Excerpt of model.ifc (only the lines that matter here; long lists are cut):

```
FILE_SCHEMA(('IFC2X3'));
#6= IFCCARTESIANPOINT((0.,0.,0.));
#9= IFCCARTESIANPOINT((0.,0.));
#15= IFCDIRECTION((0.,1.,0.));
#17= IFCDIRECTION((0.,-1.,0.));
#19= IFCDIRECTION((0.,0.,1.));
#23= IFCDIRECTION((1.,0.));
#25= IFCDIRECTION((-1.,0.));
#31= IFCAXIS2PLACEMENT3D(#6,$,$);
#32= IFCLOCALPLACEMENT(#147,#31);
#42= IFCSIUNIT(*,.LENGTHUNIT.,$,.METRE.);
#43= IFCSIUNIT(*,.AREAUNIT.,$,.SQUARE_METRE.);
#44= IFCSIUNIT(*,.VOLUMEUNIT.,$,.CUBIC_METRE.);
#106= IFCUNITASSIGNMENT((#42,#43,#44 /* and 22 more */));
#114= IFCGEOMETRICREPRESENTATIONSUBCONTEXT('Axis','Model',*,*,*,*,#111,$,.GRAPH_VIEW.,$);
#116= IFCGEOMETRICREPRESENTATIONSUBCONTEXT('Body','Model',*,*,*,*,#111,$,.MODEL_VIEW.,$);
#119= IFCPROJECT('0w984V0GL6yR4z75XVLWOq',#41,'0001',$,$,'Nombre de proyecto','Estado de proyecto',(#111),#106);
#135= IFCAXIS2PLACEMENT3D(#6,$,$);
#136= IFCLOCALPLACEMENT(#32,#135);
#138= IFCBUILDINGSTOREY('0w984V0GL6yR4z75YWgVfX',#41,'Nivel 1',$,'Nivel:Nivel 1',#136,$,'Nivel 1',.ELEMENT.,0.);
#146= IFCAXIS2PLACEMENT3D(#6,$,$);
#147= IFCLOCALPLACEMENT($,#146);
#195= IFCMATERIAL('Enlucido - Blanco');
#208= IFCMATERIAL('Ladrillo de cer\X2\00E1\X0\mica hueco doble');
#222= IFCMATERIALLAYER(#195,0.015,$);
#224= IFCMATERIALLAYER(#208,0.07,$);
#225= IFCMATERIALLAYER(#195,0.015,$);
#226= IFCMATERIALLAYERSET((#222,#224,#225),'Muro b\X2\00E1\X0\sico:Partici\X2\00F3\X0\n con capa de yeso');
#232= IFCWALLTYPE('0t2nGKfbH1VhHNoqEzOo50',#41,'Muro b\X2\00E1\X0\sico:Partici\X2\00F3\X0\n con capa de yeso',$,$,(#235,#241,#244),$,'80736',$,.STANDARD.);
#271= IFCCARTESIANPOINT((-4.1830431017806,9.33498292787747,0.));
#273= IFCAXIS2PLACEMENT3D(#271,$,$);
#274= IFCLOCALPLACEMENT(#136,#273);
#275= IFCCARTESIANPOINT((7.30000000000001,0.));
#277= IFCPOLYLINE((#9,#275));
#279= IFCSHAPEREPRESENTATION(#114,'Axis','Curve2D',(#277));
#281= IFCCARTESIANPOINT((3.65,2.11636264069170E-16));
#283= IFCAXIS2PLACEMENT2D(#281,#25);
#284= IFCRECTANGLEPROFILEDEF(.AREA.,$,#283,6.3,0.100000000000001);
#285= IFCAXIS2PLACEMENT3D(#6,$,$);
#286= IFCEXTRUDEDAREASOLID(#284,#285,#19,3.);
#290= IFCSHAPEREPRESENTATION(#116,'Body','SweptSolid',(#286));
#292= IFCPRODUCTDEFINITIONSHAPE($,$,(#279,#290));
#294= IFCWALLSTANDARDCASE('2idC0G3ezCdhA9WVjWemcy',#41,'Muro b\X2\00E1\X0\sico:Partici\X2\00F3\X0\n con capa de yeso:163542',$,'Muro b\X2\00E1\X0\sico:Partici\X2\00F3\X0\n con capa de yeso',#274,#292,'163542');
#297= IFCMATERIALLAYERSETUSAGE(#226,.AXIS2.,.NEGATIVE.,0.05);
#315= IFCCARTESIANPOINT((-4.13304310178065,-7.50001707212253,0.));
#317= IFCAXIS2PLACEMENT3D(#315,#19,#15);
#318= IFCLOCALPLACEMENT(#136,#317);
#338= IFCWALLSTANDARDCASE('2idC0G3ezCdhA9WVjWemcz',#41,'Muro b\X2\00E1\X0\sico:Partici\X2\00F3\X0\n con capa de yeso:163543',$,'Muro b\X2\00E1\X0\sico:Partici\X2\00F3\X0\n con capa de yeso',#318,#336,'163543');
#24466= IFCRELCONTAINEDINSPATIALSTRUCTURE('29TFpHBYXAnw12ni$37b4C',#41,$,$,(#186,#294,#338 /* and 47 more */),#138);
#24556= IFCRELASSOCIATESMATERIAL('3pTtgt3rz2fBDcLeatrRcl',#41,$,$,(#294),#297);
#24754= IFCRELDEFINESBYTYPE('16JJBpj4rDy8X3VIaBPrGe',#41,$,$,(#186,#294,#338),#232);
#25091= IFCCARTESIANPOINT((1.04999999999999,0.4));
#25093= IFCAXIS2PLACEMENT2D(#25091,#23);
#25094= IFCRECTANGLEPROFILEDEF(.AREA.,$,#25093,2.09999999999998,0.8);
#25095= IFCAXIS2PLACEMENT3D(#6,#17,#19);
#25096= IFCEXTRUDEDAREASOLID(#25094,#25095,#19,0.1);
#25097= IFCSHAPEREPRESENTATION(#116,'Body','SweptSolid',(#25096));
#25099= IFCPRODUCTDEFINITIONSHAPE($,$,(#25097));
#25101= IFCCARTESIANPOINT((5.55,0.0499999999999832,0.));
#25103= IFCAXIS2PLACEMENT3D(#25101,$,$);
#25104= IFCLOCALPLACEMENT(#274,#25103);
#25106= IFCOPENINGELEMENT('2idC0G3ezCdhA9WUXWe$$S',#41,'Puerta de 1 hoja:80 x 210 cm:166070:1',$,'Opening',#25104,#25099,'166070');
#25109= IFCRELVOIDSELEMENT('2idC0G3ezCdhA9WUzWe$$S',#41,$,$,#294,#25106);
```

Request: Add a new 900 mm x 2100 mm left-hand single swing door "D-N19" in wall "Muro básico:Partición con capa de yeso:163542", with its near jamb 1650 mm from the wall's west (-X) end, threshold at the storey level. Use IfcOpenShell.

```python
import numpy as np
import ifcopenshell
import ifcopenshell.api.feature
import ifcopenshell.api.geometry
import ifcopenshell.api.root
import ifcopenshell.api.spatial
import ifcopenshell.api.type
import ifcopenshell.geom
import ifcopenshell.util.element
import ifcopenshell.util.placement
import ifcopenshell.util.representation
import ifcopenshell.util.shape
import ifcopenshell.util.unit

model = ifcopenshell.open("model.ifc")
unit_scale = ifcopenshell.util.unit.calculate_unit_scale(model)
settings = ifcopenshell.geom.settings()


def volume(element):
    """Net volume in cubic metres, openings subtracted."""
    shape = ifcopenshell.geom.create_shape(settings, element)
    return ifcopenshell.util.shape.get_volume(shape.geometry)


wall = model.by_guid("2idC0G3ezCdhA9WVjWemcy")
storey = ifcopenshell.util.element.get_container(wall, ifc_class="IfcBuildingStorey")
context = ifcopenshell.util.representation.get_context(model, "Model", "Body", "MODEL_VIEW")
before = volume(wall)

width, height, from_end, sill = 0.9, 2.1, 1.65, 0.0  # metres

# The wall runs along its own X axis, and the end named is its -X end.
wall_shape = ifcopenshell.geom.create_shape(settings, wall)
x, y, z = ifcopenshell.util.shape.get_vertices(wall_shape.geometry).T
start = x.min() + from_end
face, thickness = float(y.min()), float(y.max() - y.min())
wall_matrix = ifcopenshell.util.placement.get_local_placement(wall.ObjectPlacement)
level = ifcopenshell.util.placement.get_local_placement(storey.ObjectPlacement)[2, 3]


def in_wall(x, y):
    """Placement at x, y metres in the wall's axes, at sill height."""
    matrix = wall_matrix.copy()
    matrix[:, 3] = wall_matrix @ np.array([x / unit_scale, y / unit_scale, 0.0, 1.0])
    matrix[2, 3] = level + sill / unit_scale
    return matrix


# Opening: a box that overshoots both wall faces by 50 mm.
opening = ifcopenshell.api.root.create_entity(model, ifc_class="IfcOpeningElement")
box = ifcopenshell.api.geometry.add_wall_representation(
    model, context=context, length=width, height=height, thickness=thickness + 0.1
)
ifcopenshell.api.geometry.assign_representation(model, product=opening, representation=box)
ifcopenshell.api.geometry.edit_object_placement(model, product=opening, matrix=in_wall(start, face - 0.05), is_si=False)
ifcopenshell.api.feature.add_feature(model, feature=opening, element=wall)

door = ifcopenshell.api.root.create_entity(model, ifc_class="IfcDoor", name="D-N19")
door.OverallWidth, door.OverallHeight = width / unit_scale, height / unit_scale
body = ifcopenshell.api.geometry.add_door_representation(
    model,
    context=context,
    overall_width=door.OverallWidth,
    overall_height=door.OverallHeight,
    operation_type="SINGLE_SWING_LEFT",
    lining_properties={"LiningDepth": thickness / unit_scale, "ThresholdDepth": thickness / unit_scale},
)
ifcopenshell.api.geometry.assign_representation(model, product=door, representation=body)
ifcopenshell.api.spatial.assign_container(model, products=[door], relating_structure=storey)
fills = ifcopenshell.api.feature.add_filling(model, opening=opening, element=door)
fills.OwnerHistory = door.OwnerHistory  # required in IFC2X3

# IFC2X3 keeps the operation on the door style.
style = ifcopenshell.api.root.create_entity(model, ifc_class="IfcDoorStyle", name="D-N19")
style.OperationType, style.ConstructionType = "SINGLE_SWING_LEFT", "NOTDEFINED"
style.ParameterTakesPrecedence = style.Sizeable = False
ifcopenshell.api.type.assign_type(model, related_objects=[door], relating_type=style)

# The lining spans the wall, so the door starts at the wall face.
ifcopenshell.api.geometry.edit_object_placement(model, product=door, matrix=in_wall(start, face), is_si=False)

after = volume(wall)

print(f"wall volume {before:.3f} -> {after:.3f} m3")

model.write("model_v2.ifc")
```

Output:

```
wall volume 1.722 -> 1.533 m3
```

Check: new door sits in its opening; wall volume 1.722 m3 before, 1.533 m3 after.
